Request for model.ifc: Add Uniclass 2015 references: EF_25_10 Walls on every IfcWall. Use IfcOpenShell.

First a look at what the model holds.

```python
import ifcopenshell

model = ifcopenshell.open("model.ifc")
print(model.schema)
print("classifications:", [c.Name for c in model.by_type("IfcClassification")])
for ifc_class in ("IfcDoor", "IfcRoof", "IfcStair", "IfcWall", "IfcWindow"):
    print(ifc_class, len(model.by_type(ifc_class)))
```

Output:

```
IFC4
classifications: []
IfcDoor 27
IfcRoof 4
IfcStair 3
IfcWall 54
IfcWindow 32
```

```python
import ifcopenshell
import ifcopenshell.api.classification

model = ifcopenshell.open("model.ifc")

system = ifcopenshell.api.classification.add_classification(model, classification="Uniclass 2015")

codes = {
    "IfcWall": ("EF_25_10", "Walls"),
}
for ifc_class, (code, name) in codes.items():
    products = model.by_type(ifc_class)
    ifcopenshell.api.classification.add_reference(
        model, products=products, classification=system, identification=code, name=name
    )
    print(code, len(products))

model.write("model-out.ifc")
```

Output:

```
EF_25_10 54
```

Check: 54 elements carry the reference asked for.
